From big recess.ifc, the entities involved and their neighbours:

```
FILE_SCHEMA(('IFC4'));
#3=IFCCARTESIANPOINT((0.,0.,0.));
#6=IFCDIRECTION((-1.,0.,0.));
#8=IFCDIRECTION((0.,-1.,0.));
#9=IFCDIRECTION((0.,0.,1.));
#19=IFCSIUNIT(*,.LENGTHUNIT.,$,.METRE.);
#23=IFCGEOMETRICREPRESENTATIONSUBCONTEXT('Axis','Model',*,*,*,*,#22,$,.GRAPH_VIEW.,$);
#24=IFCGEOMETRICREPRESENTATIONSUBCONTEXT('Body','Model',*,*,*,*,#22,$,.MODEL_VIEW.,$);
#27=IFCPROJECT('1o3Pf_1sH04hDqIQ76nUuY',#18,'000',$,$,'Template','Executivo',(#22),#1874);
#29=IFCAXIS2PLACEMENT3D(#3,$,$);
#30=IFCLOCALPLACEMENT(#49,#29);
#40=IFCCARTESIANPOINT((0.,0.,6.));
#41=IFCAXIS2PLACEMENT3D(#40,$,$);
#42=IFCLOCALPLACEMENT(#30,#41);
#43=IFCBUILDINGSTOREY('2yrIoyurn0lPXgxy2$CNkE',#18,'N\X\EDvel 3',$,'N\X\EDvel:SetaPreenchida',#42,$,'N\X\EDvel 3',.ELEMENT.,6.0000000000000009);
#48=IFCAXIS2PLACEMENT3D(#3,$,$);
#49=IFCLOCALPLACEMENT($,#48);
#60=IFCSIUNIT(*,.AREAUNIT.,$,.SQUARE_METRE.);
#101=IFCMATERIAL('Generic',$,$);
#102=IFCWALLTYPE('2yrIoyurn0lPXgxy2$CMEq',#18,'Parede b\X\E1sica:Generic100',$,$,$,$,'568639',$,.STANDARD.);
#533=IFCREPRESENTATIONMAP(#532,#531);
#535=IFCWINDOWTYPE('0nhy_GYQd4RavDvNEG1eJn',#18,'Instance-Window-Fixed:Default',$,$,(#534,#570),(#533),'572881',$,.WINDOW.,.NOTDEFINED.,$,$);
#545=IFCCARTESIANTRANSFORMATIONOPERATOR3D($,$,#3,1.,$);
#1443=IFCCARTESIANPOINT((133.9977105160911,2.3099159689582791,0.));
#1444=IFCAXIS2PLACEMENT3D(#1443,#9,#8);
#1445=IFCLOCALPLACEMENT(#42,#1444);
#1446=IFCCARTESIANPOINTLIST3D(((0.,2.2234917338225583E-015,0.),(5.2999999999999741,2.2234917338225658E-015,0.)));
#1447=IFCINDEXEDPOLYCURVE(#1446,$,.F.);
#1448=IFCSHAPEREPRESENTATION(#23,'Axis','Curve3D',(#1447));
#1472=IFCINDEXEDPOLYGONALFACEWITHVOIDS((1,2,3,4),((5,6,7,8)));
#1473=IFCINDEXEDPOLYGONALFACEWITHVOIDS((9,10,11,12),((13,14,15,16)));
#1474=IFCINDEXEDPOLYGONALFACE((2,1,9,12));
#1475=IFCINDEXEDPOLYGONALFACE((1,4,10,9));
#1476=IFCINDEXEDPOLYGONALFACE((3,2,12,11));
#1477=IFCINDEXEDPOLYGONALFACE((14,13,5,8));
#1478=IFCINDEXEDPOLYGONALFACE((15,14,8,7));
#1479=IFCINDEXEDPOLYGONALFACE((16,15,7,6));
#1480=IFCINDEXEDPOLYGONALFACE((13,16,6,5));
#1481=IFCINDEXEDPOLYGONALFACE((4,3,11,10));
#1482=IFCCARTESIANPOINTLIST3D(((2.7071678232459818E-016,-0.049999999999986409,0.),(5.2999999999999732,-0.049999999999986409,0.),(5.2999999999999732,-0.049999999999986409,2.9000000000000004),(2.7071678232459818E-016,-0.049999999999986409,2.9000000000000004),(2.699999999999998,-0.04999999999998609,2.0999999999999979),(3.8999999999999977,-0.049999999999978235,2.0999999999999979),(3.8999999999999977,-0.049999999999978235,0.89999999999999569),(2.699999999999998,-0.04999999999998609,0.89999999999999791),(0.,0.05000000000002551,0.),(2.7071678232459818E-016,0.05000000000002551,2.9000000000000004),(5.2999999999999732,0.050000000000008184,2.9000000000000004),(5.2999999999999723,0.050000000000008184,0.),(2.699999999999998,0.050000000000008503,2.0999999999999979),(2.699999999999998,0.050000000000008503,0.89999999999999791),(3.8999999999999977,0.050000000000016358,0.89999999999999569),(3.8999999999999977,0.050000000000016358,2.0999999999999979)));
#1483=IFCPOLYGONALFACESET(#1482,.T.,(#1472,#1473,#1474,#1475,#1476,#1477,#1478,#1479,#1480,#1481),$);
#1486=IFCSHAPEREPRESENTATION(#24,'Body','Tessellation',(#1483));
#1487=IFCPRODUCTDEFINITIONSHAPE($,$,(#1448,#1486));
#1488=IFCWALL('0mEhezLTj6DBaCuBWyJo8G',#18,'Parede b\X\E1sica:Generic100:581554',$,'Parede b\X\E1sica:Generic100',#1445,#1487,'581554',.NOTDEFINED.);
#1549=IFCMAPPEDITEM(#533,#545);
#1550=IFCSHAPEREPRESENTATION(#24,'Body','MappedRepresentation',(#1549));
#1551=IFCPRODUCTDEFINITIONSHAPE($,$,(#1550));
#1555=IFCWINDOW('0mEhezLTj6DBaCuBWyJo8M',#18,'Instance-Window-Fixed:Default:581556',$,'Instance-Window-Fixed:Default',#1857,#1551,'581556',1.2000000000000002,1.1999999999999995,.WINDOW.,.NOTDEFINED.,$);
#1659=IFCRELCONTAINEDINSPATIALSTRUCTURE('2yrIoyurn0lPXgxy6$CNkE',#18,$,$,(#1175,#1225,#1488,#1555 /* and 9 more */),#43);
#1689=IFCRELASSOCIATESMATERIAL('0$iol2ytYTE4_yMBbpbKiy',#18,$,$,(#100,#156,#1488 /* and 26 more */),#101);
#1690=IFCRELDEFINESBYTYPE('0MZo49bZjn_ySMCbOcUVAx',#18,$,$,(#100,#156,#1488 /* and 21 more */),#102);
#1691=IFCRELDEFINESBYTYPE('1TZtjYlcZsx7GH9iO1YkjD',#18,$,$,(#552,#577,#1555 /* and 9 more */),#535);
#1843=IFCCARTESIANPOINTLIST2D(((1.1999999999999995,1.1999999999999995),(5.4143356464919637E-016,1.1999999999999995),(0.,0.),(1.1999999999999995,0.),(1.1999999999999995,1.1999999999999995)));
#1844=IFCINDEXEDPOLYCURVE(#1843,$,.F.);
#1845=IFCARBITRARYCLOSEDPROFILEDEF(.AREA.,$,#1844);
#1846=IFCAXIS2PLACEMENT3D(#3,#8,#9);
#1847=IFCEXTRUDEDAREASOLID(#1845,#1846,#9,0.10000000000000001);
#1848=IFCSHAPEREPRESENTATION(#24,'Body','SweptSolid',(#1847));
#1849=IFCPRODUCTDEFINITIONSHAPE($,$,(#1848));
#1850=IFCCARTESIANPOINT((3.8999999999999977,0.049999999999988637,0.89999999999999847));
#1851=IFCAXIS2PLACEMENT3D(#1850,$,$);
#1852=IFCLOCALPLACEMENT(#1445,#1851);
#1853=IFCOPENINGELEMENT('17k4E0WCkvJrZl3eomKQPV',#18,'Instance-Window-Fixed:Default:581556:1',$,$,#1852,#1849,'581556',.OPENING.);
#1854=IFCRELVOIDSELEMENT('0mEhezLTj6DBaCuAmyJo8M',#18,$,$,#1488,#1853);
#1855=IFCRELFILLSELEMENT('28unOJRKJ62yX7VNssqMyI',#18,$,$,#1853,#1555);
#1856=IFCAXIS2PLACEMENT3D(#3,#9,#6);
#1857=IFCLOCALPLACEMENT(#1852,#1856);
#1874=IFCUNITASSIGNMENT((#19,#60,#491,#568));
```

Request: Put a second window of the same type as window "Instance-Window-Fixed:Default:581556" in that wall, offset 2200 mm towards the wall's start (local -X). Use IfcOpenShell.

```python
import ifcopenshell
import ifcopenshell.api.feature
import ifcopenshell.api.geometry
import ifcopenshell.api.root
import ifcopenshell.geom
import ifcopenshell.util.element
import ifcopenshell.util.placement
import ifcopenshell.util.shape
import ifcopenshell.util.unit

model = ifcopenshell.open("big recess.ifc")
unit_scale = ifcopenshell.util.unit.calculate_unit_scale(model)
settings = ifcopenshell.geom.settings()


def volume(element):
    """Net volume in cubic metres, openings subtracted."""
    shape = ifcopenshell.geom.create_shape(settings, element)
    return ifcopenshell.util.shape.get_volume(shape.geometry)


def reuse_history(source, copy):
    """copy_class also copies each property set's owner history, people and application; keep the originals."""
    for rel in copy.IsDefinedBy:
        if rel.is_a("IfcRelDefinesByProperties") and (history := rel.RelatingPropertyDefinition.OwnerHistory):
            rel.RelatingPropertyDefinition.OwnerHistory = source.OwnerHistory
            ifcopenshell.util.element.remove_deep2(model, history)


window = model.by_id(1555)
opening = window.FillsVoids[0].RelatingOpeningElement
wall = opening.VoidsElements[0].RelatingBuildingElement
before = volume(wall)
shift = ifcopenshell.util.placement.get_local_placement(wall.ObjectPlacement)[:3, 0] * -2.2 / unit_scale

# copy_class copies the void relationship, type, container and properties, but no geometry.
new_opening = ifcopenshell.api.root.copy_class(model, product=opening)
new_opening.Representation = ifcopenshell.util.element.copy_deep(
    model, opening.Representation, exclude=["IfcGeometricRepresentationContext", "IfcRepresentationMap"]
)
new_opening.Name = "Instance-Window-Fixed:Default"
new_opening.Tag = None
new_window = ifcopenshell.api.root.copy_class(model, product=window)
new_window.Representation = ifcopenshell.util.element.copy_deep(
    model, window.Representation, exclude=["IfcGeometricRepresentationContext", "IfcRepresentationMap"]
)
new_window.Name = "Instance-Window-Fixed:Default"
new_window.Tag = None
reuse_history(window, new_window)
ifcopenshell.api.feature.add_filling(model, opening=new_opening, element=new_window)

for old, new in ((opening, new_opening), (window, new_window)):
    matrix = ifcopenshell.util.placement.get_local_placement(old.ObjectPlacement)
    matrix[:3, 3] += shift
    ifcopenshell.api.geometry.edit_object_placement(model, product=new, matrix=matrix, is_si=False)

after = volume(wall)

print(f"wall volume {before:.3f} -> {after:.3f} m3")

model.write("big recess_v2.ifc")
```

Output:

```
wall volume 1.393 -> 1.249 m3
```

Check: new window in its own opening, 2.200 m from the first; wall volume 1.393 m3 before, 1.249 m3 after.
